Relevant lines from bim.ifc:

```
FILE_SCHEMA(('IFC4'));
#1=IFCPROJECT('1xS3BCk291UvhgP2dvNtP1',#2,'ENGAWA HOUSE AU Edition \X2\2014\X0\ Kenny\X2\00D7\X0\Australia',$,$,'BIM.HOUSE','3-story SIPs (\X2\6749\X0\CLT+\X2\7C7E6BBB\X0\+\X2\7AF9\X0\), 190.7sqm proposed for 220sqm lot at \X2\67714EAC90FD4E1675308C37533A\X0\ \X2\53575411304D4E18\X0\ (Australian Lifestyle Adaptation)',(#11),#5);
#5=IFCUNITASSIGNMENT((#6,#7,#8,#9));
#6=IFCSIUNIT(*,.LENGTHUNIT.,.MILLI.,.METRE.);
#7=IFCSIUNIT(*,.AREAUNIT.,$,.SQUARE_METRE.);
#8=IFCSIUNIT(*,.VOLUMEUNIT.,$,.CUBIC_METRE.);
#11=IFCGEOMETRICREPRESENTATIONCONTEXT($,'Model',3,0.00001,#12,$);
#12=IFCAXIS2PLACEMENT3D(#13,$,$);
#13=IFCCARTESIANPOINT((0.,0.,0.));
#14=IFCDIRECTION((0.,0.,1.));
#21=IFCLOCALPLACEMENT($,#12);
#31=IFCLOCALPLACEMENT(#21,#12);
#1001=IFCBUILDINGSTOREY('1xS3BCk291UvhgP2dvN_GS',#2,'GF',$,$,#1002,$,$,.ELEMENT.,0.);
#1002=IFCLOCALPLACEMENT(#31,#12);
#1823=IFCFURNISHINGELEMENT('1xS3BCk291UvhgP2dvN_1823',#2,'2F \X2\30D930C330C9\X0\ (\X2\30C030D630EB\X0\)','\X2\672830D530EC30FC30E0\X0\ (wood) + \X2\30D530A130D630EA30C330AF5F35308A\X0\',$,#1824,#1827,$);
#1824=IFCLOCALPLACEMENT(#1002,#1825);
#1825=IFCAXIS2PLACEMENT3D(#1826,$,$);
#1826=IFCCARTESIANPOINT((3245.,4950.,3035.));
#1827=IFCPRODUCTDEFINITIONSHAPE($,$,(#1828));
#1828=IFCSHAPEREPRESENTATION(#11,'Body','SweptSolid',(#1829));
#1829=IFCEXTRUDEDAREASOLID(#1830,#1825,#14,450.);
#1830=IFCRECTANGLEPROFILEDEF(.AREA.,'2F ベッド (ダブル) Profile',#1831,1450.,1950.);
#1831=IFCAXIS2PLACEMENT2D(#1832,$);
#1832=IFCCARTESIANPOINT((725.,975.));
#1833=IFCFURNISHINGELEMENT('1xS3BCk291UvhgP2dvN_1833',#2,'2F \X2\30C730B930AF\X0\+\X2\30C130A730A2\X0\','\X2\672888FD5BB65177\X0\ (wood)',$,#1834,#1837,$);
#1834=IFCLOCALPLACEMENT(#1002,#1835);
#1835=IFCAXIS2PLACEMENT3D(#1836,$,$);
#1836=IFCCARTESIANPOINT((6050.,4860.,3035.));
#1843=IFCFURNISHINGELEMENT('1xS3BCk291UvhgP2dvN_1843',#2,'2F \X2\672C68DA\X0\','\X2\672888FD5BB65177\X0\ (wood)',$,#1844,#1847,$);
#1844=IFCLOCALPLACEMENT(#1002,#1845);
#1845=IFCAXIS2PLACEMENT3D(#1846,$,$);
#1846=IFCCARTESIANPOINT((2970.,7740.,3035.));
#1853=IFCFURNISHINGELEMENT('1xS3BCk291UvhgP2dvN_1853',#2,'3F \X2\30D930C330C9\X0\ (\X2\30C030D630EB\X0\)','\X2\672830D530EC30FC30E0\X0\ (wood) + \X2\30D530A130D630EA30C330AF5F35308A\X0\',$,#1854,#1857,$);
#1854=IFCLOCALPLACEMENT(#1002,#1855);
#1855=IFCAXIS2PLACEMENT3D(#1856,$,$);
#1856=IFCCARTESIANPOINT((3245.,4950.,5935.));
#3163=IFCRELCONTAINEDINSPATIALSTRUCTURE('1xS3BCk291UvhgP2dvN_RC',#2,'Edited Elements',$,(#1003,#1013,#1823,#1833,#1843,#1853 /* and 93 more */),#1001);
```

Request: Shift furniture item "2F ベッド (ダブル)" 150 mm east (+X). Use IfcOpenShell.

```python
import ifcopenshell
import ifcopenshell.api.geometry
import ifcopenshell.util.placement
import ifcopenshell.util.unit

model = ifcopenshell.open("bim.ifc")
unit_scale = ifcopenshell.util.unit.calculate_unit_scale(model)

item = model.by_id(1823)
matrix = ifcopenshell.util.placement.get_local_placement(item.ObjectPlacement)
matrix[0, 3] += 0.15 / unit_scale
ifcopenshell.api.geometry.edit_object_placement(model, product=item, matrix=matrix, is_si=False)

print(ifcopenshell.util.placement.get_local_placement(item.ObjectPlacement).round(3) + 0.0)

model.write("bim-out.ifc")
```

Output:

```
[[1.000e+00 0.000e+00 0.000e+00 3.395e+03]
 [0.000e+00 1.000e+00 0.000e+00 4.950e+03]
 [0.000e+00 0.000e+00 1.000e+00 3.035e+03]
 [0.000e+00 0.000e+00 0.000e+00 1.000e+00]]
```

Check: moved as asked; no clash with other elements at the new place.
